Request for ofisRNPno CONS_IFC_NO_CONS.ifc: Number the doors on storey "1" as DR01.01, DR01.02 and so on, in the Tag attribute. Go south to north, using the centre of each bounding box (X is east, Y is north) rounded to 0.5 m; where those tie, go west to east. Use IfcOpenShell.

First a look at what the model holds.

```python
import ifcopenshell
import ifcopenshell.util.element
import ifcopenshell.util.placement

model = ifcopenshell.open("ofisRNPno CONS_IFC_NO_CONS.ifc")
print(model.schema)
storey = next(s for s in model.by_type("IfcBuildingStorey") if s.Name == "1")
doors = [e for e in ifcopenshell.util.element.get_decomposition(storey) if e.is_a("IfcDoor")]
for e in sorted(doors, key=lambda e: e.id()):
    origin = ifcopenshell.util.placement.get_local_placement(e.ObjectPlacement)[:3, 3]
    print(e.id(), e.Tag, e.Name, origin.round(2) + 0.0, sep=" | ")
```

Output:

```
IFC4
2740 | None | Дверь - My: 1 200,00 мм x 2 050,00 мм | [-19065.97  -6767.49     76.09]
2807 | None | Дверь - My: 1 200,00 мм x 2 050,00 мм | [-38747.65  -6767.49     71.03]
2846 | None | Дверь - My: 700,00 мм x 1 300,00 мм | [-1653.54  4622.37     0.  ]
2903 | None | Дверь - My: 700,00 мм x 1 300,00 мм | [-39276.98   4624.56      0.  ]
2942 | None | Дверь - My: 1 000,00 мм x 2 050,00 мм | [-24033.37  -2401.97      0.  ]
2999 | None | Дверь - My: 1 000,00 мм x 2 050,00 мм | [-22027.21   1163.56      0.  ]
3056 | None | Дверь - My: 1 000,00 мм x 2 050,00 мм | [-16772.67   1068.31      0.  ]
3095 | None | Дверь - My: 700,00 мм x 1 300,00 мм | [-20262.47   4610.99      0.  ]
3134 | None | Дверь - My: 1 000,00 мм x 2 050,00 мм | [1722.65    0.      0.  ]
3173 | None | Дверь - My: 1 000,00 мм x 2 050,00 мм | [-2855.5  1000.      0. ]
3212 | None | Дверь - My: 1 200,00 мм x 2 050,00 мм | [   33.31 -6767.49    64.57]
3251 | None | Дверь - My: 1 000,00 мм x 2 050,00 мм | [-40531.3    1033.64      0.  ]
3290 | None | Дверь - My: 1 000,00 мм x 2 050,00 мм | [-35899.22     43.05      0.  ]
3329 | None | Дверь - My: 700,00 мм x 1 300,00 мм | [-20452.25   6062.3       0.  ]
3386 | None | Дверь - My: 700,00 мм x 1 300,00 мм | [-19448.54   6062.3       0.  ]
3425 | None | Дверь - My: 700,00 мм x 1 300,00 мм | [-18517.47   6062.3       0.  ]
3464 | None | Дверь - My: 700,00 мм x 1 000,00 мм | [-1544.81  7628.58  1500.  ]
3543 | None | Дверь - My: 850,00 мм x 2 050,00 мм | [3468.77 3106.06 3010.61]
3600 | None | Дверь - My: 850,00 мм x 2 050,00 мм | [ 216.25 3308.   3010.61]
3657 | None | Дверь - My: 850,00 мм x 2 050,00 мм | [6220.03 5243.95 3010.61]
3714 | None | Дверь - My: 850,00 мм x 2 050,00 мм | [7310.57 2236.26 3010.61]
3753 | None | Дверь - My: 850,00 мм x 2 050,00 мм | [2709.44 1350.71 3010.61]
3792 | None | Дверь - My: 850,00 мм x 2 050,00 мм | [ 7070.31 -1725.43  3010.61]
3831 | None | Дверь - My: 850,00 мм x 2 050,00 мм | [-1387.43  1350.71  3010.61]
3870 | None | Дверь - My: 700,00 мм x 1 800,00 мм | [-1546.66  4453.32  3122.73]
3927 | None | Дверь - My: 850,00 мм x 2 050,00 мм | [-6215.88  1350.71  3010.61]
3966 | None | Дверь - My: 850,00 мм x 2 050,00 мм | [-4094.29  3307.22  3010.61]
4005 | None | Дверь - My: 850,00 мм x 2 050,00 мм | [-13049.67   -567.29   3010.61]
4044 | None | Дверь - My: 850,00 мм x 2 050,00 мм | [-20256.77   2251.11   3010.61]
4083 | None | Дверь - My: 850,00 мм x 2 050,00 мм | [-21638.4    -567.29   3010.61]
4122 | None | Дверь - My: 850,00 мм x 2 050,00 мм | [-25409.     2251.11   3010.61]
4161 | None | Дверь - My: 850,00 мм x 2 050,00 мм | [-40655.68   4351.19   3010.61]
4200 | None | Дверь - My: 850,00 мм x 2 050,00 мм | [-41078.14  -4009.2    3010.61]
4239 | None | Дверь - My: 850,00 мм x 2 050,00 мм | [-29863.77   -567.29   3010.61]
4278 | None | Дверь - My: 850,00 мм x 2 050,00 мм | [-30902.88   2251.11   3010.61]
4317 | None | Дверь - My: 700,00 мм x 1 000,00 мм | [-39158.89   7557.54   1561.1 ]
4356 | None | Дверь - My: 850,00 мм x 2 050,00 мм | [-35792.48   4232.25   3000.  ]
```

```python
import ifcopenshell
import ifcopenshell.geom
import ifcopenshell.util.element
import ifcopenshell.util.shape

model = ifcopenshell.open("ofisRNPno CONS_IFC_NO_CONS.ifc")
settings = ifcopenshell.geom.settings()
settings.set("use-world-coords", True)


def centre(element):
    shape = ifcopenshell.geom.create_shape(settings, element)
    return ifcopenshell.util.shape.get_bbox_centroid(shape.geometry)


storey = next(s for s in model.by_type("IfcBuildingStorey") if s.Name == "1")
doors = [e for e in ifcopenshell.util.element.get_decomposition(storey) if e.is_a("IfcDoor")]

# Insertion points can sit at a corner or the storey origin, so sort by the geometry (in metres).
centres = {e: centre(e) for e in doors}
doors.sort(key=lambda e: (round(centres[e][1] / 0.5), centres[e][0]))

for i, e in enumerate(doors, start=1):
    number = f"DR01.{i:02d}"
    e.Tag = number
    print(e.id(), number)

model.write("ofisRNPno CONS_IFC_NO_CONS_edited.ifc")
```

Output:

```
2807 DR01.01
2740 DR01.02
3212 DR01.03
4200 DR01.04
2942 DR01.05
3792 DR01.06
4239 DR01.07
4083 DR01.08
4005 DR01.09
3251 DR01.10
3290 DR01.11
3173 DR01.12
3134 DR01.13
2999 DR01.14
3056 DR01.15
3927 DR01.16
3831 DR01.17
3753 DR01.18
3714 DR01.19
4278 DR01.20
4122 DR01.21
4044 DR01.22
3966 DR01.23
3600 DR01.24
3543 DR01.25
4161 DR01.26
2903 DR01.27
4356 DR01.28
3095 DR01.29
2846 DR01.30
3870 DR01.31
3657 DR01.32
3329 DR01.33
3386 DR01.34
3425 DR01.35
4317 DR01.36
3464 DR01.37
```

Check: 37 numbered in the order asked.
